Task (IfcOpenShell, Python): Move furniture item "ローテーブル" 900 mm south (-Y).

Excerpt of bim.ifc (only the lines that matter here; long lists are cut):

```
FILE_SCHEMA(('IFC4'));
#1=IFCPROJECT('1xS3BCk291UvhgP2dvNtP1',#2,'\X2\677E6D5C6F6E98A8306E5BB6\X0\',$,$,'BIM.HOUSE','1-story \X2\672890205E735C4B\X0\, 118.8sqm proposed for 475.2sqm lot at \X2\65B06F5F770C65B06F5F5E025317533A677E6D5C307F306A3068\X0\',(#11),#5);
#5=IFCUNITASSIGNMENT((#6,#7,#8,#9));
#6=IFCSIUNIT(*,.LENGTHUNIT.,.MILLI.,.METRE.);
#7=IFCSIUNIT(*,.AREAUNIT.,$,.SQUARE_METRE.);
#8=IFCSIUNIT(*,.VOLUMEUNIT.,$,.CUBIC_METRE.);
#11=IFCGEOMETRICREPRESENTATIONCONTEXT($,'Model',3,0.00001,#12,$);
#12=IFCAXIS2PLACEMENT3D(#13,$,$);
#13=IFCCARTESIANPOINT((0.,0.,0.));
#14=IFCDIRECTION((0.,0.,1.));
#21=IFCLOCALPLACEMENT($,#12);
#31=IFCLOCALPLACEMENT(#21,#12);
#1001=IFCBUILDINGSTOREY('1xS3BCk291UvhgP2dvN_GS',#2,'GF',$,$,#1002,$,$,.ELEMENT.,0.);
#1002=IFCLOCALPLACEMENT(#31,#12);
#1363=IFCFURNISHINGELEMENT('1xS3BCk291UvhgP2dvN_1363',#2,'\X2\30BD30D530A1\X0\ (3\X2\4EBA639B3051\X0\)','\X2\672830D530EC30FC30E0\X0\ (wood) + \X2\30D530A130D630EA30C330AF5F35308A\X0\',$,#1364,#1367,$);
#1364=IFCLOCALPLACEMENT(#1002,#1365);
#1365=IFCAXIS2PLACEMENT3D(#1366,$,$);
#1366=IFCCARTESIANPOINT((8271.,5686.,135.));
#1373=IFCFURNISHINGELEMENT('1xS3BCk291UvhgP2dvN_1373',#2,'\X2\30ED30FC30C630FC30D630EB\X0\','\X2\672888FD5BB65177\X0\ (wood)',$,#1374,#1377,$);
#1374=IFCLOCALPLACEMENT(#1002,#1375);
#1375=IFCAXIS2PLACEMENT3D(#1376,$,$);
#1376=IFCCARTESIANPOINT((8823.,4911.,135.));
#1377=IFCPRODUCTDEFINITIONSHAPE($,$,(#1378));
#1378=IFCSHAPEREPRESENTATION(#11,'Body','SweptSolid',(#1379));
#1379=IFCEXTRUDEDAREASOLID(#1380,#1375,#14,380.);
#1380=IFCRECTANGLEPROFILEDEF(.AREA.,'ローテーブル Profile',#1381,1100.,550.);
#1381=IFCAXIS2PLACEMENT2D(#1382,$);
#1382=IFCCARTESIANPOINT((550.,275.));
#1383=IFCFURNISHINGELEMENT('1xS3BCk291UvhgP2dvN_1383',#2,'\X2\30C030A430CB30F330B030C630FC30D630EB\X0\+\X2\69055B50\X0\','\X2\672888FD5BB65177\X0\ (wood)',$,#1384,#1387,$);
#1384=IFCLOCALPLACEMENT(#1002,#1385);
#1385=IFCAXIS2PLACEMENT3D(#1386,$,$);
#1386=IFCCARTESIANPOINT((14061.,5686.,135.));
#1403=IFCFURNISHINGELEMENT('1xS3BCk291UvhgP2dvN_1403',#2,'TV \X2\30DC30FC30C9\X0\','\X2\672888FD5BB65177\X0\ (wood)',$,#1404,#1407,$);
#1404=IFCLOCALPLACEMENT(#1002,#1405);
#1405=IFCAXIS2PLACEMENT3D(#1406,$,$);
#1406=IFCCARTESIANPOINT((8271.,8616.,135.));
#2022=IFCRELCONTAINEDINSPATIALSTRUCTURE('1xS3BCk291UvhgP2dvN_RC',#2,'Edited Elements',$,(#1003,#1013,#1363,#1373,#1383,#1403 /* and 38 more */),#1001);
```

```python
import ifcopenshell
import ifcopenshell.api.geometry
import ifcopenshell.util.placement
import ifcopenshell.util.unit

model = ifcopenshell.open("bim.ifc")
unit_scale = ifcopenshell.util.unit.calculate_unit_scale(model)

item = model.by_guid("1xS3BCk291UvhgP2dvN_1373")
matrix = ifcopenshell.util.placement.get_local_placement(item.ObjectPlacement)
matrix[1, 3] -= 0.9 / unit_scale
ifcopenshell.api.geometry.edit_object_placement(model, product=item, matrix=matrix, is_si=False)

print(ifcopenshell.util.placement.get_local_placement(item.ObjectPlacement).round(3) + 0.0)

model.write("bim_rev.ifc")
```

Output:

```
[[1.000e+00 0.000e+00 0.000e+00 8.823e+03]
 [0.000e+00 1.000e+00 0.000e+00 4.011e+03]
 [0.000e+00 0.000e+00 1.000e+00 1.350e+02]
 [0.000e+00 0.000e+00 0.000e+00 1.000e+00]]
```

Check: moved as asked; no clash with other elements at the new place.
